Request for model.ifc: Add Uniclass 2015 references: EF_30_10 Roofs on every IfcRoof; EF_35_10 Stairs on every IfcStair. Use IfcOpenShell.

First a look at what the model holds.

```python
import ifcopenshell

model = ifcopenshell.open("model.ifc")
print(model.schema)
print("classifications:", [c.Name for c in model.by_type("IfcClassification")])
for ifc_class in ("IfcDoor", "IfcRoof", "IfcStair", "IfcWall", "IfcWindow"):
    print(ifc_class, len(model.by_type(ifc_class)))
```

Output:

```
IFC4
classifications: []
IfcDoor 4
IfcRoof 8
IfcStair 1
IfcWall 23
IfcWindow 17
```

```python
import ifcopenshell
import ifcopenshell.api.classification

model = ifcopenshell.open("model.ifc")

system = ifcopenshell.api.classification.add_classification(model, classification="Uniclass 2015")

codes = {
    "IfcRoof": ("EF_30_10", "Roofs"),
    "IfcStair": ("EF_35_10", "Stairs"),
}
for ifc_class, (code, name) in codes.items():
    products = model.by_type(ifc_class)
    ifcopenshell.api.classification.add_reference(
        model, products=products, classification=system, identification=code, name=name
    )
    print(code, len(products))

model.write("model_edited.ifc")
```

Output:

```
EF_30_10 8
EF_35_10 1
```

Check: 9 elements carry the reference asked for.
